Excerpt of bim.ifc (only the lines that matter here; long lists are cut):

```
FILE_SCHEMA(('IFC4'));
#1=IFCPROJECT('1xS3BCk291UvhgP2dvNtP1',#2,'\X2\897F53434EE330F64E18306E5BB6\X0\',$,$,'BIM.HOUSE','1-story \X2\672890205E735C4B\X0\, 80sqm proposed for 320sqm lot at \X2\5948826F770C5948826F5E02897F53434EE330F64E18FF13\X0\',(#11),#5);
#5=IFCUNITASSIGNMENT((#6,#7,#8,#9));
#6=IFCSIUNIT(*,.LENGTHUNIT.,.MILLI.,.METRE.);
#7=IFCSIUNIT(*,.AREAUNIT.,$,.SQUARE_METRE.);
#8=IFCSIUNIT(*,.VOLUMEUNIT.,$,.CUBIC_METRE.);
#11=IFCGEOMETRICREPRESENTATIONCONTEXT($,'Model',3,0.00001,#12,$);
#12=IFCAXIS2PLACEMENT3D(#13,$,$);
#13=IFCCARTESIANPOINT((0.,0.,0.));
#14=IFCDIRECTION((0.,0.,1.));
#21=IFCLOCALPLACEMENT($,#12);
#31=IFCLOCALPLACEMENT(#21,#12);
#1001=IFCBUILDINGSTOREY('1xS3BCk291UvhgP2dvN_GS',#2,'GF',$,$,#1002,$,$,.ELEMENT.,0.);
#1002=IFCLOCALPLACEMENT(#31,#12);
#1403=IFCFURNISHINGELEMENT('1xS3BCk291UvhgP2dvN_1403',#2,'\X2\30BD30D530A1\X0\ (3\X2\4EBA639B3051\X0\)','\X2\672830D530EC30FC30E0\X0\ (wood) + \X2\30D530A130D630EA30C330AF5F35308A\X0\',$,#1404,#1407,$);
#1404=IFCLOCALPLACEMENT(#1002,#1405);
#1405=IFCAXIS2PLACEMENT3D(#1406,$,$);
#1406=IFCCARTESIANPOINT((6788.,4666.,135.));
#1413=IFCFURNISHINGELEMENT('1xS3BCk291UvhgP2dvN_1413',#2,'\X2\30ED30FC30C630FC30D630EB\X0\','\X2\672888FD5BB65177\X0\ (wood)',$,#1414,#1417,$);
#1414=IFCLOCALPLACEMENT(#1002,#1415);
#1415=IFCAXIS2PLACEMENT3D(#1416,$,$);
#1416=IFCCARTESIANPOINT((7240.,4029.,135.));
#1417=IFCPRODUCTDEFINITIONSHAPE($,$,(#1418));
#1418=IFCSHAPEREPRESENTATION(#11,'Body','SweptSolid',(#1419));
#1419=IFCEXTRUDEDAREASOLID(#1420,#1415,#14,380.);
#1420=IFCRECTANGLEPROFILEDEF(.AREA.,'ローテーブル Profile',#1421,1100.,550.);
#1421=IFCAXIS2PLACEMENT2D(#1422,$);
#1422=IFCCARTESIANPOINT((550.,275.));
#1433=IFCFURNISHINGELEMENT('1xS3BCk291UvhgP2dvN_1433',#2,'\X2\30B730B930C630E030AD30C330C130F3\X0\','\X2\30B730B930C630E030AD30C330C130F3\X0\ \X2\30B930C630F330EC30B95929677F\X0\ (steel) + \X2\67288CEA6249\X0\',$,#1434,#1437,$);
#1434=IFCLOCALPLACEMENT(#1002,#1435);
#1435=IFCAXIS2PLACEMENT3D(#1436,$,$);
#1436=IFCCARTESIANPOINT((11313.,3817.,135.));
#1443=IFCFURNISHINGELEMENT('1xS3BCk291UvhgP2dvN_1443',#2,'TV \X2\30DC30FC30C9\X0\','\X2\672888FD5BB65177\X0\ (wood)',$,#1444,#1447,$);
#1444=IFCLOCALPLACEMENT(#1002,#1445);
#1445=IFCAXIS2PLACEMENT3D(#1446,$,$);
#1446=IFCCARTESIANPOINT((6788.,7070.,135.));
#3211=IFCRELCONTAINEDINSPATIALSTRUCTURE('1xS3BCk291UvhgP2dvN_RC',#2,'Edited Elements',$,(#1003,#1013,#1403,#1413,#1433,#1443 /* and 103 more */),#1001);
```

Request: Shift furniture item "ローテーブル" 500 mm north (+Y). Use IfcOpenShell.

```python
import ifcopenshell
import ifcopenshell.api.geometry
import ifcopenshell.util.placement

model = ifcopenshell.open("bim.ifc")

item = model.by_guid("1xS3BCk291UvhgP2dvN_1413")
matrix = ifcopenshell.util.placement.get_local_placement(item.ObjectPlacement)
matrix[1, 3] += 500.0
ifcopenshell.api.geometry.edit_object_placement(model, product=item, matrix=matrix, is_si=False)

print(ifcopenshell.util.placement.get_local_placement(item.ObjectPlacement).round(3) + 0.0)

model.write("bim_edited.ifc")
```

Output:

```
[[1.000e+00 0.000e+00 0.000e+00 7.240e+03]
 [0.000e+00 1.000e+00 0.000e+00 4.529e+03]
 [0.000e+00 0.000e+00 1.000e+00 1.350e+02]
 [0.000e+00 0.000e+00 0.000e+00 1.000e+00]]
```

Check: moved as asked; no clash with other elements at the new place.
